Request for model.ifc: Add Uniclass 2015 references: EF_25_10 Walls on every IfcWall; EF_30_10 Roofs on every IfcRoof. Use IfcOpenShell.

First a look at what the model holds.

```python
import ifcopenshell

model = ifcopenshell.open("model.ifc")
print(model.schema)
print("classifications:", [c.Name for c in model.by_type("IfcClassification")])
for ifc_class in ("IfcDoor", "IfcRoof", "IfcStair", "IfcWall", "IfcWindow"):
    print(ifc_class, len(model.by_type(ifc_class)))
```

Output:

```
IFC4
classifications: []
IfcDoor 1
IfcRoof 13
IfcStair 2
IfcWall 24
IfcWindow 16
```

```python
import ifcopenshell
import ifcopenshell.api.classification

model = ifcopenshell.open("model.ifc")

system = ifcopenshell.api.classification.add_classification(model, classification="Uniclass 2015")

codes = {
    "IfcWall": ("EF_25_10", "Walls"),
    "IfcRoof": ("EF_30_10", "Roofs"),
}
for ifc_class, (code, name) in codes.items():
    products = model.by_type(ifc_class)
    ifcopenshell.api.classification.add_reference(
        model, products=products, classification=system, identification=code, name=name
    )
    print(code, len(products))

model.write("model-out.ifc")
```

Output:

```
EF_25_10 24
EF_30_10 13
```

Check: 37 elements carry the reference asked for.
